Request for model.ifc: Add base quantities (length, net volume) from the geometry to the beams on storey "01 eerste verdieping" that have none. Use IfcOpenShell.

First a look at what the model holds.

```python
import ifcopenshell
import ifcopenshell.util.element
import ifcopenshell.util.unit

model = ifcopenshell.open("model.ifc")
print(model.schema)
for unit_type in ("LENGTHUNIT", "AREAUNIT", "VOLUMEUNIT"):
    print(unit_type, ifcopenshell.util.unit.calculate_unit_scale(model, unit_type))
storey = next(s for s in model.by_type("IfcBuildingStorey") if s.Name == "01 eerste verdieping")
beams = [e for e in ifcopenshell.util.element.get_decomposition(storey) if e.is_a("IfcBeam")]
for e in sorted(beams, key=lambda e: e.id()):
    print(e.id(), e.is_a(), e.Name, list(ifcopenshell.util.element.get_psets(e, qtos_only=True)), sep=" | ")
```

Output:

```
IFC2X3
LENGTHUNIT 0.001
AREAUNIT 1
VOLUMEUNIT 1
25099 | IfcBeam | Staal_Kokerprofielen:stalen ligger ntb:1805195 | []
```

```python
import ifcopenshell
import ifcopenshell.api.pset
import ifcopenshell.geom
import ifcopenshell.util.element
import ifcopenshell.util.shape
import ifcopenshell.util.unit

model = ifcopenshell.open("model.ifc")
unit_scale = ifcopenshell.util.unit.calculate_unit_scale(model)
volume_scale = ifcopenshell.util.unit.calculate_unit_scale(model, "VOLUMEUNIT")
settings = ifcopenshell.geom.settings()

storey = next(s for s in model.by_type("IfcBuildingStorey") if s.Name == "01 eerste verdieping")
beams = [e for e in ifcopenshell.util.element.get_decomposition(storey) if e.is_a("IfcBeam")]

for e in sorted(beams, key=lambda e: e.id()):
    if ifcopenshell.util.element.get_psets(e, qtos_only=True, should_inherit=False):
        continue
    # Geometry comes back in metres, in the element's own axes.
    shape = ifcopenshell.geom.create_shape(settings, e)
    values = {
        "Length": ifcopenshell.util.shape.get_max_xyz(shape.geometry) / unit_scale,
        "NetVolume": ifcopenshell.util.shape.get_volume(shape.geometry) / volume_scale,
    }
    qto = ifcopenshell.api.pset.add_qto(model, product=e, name="BaseQuantities")
    ifcopenshell.api.pset.edit_qto(model, qto=qto, properties=values)
    print(e.id(), {k: round(v, 3) for k, v in values.items()})

model.write("model_edited.ifc")
```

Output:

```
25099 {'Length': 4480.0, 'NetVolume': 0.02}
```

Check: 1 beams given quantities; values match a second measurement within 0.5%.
